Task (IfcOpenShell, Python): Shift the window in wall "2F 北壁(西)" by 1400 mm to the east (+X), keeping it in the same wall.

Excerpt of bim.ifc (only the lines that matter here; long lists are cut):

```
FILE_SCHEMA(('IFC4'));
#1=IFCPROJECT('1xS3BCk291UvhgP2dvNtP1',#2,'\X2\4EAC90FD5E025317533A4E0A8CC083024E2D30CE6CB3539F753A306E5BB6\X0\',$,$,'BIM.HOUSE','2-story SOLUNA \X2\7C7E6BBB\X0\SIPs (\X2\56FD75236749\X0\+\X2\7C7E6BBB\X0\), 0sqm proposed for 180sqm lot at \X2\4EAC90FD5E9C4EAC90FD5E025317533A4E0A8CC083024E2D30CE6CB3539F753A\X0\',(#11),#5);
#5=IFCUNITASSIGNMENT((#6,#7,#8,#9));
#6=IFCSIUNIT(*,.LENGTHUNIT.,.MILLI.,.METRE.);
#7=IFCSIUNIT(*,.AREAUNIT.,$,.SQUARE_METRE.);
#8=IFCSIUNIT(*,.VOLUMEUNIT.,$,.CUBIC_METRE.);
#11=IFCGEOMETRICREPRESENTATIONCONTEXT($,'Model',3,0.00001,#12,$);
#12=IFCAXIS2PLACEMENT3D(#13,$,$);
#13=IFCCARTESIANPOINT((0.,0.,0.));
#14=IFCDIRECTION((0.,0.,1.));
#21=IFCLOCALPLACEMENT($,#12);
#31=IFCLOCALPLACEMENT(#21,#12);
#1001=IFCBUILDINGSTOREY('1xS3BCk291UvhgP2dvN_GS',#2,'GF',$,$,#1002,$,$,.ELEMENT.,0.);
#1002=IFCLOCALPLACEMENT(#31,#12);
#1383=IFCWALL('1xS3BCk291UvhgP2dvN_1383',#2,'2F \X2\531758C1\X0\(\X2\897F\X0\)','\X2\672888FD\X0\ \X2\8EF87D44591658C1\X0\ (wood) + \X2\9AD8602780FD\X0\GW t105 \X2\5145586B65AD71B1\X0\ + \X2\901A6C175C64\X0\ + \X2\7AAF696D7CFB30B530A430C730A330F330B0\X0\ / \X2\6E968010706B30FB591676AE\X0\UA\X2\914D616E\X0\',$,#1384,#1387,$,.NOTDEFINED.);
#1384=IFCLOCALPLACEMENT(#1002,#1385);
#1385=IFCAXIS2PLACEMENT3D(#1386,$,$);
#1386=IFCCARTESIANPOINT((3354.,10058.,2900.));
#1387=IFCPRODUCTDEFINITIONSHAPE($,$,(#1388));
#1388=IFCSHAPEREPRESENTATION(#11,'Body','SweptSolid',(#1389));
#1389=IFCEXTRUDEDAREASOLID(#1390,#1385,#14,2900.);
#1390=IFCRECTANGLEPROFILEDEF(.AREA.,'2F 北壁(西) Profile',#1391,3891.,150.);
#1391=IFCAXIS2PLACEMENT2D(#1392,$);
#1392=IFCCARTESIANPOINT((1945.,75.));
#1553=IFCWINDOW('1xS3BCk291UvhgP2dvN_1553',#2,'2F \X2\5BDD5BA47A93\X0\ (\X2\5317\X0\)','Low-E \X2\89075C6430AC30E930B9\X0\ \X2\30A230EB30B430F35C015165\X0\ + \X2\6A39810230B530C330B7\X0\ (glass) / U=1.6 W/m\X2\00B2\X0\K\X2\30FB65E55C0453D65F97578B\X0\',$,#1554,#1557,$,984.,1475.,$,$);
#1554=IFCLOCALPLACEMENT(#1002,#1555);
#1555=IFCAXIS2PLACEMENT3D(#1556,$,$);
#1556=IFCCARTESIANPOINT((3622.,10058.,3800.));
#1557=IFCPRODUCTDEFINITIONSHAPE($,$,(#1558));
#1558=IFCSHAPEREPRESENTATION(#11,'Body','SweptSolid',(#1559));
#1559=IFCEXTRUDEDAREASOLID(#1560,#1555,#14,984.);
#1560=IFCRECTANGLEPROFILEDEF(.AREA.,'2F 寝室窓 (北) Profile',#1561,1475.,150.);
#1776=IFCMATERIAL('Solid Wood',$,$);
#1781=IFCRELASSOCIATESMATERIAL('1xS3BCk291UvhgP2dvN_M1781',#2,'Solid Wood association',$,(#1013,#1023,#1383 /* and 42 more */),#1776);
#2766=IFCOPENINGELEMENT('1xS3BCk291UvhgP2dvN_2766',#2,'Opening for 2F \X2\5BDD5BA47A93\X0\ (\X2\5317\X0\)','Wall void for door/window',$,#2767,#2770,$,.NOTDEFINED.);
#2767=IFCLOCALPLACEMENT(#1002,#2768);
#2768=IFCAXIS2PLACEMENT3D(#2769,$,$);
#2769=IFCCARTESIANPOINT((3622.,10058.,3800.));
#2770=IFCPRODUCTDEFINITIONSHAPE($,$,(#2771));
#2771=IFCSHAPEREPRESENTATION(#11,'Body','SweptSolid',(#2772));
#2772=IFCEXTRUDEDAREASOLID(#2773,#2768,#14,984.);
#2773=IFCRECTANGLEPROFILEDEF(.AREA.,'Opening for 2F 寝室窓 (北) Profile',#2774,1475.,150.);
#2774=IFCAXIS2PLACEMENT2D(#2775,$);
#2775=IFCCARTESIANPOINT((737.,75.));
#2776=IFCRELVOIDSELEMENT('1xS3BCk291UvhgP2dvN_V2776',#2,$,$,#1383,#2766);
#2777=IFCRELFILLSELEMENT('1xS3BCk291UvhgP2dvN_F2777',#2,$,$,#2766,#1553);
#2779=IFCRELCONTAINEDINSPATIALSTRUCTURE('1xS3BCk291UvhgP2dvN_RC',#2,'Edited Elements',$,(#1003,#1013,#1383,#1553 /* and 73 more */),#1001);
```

```python
import ifcopenshell
import ifcopenshell.api.geometry
import ifcopenshell.util.placement
import ifcopenshell.util.unit

model = ifcopenshell.open("bim.ifc")
unit_scale = ifcopenshell.util.unit.calculate_unit_scale(model)

window = model.by_id(1553)
opening = window.FillsVoids[0].RelatingOpeningElement
wall = opening.VoidsElements[0].RelatingBuildingElement

wall_matrix = ifcopenshell.util.placement.get_local_placement(wall.ObjectPlacement)
shift = wall_matrix[:3, 0] * 1.4 / unit_scale
before = ifcopenshell.util.placement.get_local_placement(window.ObjectPlacement)[:3, 3].copy()

# The window is not placed relative to its opening, so move both.
for product in (opening, window):
    matrix = ifcopenshell.util.placement.get_local_placement(product.ObjectPlacement)
    matrix[:3, 3] += shift
    ifcopenshell.api.geometry.edit_object_placement(model, product=product, matrix=matrix, is_si=False)

after = ifcopenshell.util.placement.get_local_placement(window.ObjectPlacement)[:3, 3]
print("window moved by", (after - before).round(3) + 0.0)

model.write("bim_updated.ifc")
```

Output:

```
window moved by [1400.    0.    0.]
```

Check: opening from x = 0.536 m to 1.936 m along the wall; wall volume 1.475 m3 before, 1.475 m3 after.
